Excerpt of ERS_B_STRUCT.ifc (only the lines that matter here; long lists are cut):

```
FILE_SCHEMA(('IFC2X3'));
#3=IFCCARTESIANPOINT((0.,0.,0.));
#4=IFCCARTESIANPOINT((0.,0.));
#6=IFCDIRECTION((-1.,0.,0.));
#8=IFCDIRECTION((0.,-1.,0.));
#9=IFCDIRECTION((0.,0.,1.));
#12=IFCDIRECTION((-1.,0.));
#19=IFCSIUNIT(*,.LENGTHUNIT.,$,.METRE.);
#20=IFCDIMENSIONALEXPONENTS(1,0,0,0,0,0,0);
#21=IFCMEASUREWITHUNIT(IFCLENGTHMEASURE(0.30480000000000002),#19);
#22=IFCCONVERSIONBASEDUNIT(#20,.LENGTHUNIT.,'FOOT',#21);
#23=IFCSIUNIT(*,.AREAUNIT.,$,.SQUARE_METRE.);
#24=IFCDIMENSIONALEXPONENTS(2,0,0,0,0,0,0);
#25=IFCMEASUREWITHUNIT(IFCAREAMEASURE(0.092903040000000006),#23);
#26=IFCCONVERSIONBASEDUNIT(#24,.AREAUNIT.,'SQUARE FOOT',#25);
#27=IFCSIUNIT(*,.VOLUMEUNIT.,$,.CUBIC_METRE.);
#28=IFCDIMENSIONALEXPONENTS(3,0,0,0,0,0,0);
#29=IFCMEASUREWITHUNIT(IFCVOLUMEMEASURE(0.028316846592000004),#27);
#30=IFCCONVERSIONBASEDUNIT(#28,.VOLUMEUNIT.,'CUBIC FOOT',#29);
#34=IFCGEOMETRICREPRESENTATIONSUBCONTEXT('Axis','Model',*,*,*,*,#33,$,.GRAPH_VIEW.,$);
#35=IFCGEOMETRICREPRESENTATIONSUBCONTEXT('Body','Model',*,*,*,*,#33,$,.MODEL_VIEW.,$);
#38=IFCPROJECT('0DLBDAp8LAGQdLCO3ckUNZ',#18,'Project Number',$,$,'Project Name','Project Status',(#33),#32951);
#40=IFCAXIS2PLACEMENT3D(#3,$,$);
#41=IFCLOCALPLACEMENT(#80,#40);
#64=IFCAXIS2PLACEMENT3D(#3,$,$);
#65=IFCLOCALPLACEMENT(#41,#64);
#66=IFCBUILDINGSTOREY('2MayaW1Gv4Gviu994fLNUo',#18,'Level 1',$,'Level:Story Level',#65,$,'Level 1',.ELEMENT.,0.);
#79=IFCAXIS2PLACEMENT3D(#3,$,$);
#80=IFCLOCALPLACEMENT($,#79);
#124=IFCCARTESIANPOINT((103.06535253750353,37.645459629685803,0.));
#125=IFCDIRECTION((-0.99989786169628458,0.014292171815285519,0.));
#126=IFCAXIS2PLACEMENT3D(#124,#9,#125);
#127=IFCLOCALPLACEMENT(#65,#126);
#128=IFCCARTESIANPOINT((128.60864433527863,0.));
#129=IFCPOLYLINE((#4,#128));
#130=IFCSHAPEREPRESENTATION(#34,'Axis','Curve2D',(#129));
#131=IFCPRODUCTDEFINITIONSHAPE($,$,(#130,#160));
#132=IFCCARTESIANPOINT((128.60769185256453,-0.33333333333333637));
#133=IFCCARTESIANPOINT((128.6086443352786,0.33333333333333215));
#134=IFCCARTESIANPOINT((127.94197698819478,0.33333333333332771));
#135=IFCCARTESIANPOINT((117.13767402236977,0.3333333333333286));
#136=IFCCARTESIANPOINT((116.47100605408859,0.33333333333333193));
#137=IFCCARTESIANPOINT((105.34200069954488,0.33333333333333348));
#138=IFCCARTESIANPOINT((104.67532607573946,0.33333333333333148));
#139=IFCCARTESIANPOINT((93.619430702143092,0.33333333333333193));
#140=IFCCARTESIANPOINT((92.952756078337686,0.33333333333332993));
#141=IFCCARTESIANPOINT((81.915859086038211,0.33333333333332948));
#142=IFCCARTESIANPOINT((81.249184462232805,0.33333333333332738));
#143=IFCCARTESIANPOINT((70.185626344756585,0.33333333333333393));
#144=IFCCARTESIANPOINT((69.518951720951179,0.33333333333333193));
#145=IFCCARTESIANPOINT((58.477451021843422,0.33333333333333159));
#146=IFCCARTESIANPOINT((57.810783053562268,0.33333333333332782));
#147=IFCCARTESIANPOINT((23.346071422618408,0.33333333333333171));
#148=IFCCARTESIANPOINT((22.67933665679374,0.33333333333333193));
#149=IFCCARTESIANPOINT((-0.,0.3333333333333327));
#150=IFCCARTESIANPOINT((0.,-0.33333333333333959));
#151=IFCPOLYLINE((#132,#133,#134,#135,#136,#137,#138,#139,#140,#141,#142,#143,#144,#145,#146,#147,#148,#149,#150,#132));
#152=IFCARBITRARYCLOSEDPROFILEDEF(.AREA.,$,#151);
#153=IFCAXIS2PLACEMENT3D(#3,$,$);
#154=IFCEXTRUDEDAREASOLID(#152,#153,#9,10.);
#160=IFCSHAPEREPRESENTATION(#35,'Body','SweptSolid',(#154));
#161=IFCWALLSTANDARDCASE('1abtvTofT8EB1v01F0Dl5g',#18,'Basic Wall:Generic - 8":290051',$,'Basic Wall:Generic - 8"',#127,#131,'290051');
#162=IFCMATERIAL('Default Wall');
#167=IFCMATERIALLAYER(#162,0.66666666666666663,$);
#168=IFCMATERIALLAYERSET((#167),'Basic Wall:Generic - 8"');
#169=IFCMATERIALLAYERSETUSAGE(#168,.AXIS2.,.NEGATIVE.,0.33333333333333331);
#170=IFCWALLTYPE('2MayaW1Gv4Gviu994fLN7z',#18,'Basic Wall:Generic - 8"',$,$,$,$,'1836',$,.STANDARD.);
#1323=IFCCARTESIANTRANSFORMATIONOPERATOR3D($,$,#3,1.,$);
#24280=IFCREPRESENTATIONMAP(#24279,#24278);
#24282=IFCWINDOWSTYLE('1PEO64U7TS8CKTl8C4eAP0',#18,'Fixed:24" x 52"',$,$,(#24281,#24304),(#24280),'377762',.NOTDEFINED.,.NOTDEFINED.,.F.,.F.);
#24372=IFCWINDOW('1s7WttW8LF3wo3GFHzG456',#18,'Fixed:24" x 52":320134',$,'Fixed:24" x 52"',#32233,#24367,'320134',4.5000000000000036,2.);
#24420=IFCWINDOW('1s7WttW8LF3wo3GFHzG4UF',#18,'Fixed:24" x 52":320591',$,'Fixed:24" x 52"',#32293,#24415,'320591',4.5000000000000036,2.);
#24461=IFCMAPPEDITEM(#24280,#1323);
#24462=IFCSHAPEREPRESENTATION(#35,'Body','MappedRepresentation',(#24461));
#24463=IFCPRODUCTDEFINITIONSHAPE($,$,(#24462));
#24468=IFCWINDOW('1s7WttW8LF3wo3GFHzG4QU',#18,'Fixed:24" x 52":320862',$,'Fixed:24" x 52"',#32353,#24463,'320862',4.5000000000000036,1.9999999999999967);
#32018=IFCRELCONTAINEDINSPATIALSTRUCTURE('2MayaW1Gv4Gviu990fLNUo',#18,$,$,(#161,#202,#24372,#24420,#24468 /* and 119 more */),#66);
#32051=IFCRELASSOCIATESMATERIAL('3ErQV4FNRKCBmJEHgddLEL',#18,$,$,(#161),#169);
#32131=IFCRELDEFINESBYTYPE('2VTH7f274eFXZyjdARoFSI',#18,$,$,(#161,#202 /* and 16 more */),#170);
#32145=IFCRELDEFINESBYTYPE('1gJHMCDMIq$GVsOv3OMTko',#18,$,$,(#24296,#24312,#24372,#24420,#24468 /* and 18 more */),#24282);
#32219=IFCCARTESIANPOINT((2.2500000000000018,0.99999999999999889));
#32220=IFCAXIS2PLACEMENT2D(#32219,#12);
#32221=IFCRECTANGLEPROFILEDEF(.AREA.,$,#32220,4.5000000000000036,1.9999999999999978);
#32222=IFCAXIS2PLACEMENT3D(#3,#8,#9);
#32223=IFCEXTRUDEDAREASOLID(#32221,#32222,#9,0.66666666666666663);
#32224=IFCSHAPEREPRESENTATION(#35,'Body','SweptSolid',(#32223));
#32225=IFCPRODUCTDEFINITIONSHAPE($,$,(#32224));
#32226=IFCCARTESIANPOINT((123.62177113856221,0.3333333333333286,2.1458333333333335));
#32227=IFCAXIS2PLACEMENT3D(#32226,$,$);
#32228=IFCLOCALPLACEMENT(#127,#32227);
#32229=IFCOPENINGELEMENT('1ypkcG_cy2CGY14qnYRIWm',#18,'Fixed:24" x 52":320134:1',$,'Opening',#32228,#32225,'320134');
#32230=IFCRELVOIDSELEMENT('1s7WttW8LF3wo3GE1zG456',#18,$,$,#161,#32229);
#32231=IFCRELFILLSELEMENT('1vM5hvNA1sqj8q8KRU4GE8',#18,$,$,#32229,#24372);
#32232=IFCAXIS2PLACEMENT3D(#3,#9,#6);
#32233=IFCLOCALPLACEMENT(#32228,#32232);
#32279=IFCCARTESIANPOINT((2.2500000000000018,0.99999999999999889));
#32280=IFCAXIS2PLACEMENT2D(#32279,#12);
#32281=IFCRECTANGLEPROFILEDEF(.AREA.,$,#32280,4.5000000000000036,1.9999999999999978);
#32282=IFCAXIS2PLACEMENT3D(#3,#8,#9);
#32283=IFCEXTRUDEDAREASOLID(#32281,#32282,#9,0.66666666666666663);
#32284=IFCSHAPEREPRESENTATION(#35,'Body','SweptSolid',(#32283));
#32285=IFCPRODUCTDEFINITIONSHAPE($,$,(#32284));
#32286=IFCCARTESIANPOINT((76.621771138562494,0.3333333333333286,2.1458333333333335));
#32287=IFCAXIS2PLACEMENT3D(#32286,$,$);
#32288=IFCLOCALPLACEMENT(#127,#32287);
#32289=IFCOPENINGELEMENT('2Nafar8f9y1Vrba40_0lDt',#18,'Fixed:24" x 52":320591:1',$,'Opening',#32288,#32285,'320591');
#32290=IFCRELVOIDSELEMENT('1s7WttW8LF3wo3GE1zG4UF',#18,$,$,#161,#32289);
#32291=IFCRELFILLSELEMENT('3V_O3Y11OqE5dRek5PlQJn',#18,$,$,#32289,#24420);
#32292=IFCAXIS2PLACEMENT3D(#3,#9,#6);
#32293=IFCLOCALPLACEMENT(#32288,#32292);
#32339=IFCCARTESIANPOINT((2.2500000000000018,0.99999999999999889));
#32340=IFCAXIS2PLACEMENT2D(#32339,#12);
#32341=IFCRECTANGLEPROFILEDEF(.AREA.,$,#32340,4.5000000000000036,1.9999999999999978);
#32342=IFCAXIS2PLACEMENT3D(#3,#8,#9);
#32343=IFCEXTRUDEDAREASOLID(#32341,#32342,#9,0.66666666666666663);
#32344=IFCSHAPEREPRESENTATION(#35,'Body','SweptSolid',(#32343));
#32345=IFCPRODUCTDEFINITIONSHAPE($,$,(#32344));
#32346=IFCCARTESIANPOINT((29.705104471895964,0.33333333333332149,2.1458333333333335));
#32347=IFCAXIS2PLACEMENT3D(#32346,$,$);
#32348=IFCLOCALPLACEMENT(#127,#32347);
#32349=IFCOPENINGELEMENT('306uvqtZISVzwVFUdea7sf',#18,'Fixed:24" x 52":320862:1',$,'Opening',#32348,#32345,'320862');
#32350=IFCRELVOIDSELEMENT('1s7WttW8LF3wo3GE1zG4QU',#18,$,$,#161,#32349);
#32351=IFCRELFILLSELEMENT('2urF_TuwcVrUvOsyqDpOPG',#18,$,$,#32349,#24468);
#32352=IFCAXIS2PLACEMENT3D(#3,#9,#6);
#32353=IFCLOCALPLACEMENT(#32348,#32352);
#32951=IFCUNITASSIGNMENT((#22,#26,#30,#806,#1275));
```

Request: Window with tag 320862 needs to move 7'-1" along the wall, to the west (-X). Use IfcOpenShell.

```python
import ifcopenshell
import ifcopenshell.api.geometry
import ifcopenshell.util.placement
import ifcopenshell.util.unit

model = ifcopenshell.open("ERS_B_STRUCT.ifc")
unit_scale = ifcopenshell.util.unit.calculate_unit_scale(model)

window = model.by_guid("1s7WttW8LF3wo3GFHzG4QU")
opening = window.FillsVoids[0].RelatingOpeningElement
wall = opening.VoidsElements[0].RelatingBuildingElement

wall_matrix = ifcopenshell.util.placement.get_local_placement(wall.ObjectPlacement)
shift = wall_matrix[:3, 0] * 85 * 0.0254 / unit_scale
before = ifcopenshell.util.placement.get_local_placement(window.ObjectPlacement)[:3, 3].copy()

# The window is placed relative to its opening, so it follows when the opening moves.
matrix = ifcopenshell.util.placement.get_local_placement(opening.ObjectPlacement)
matrix[:3, 3] += shift
ifcopenshell.api.geometry.edit_object_placement(
    model, product=opening, matrix=matrix, is_si=False, should_transform_children=True
)

after = ifcopenshell.util.placement.get_local_placement(window.ObjectPlacement)[:3, 3]
print("window moved by", (after - before).round(3) + 0.0)

model.write("ERS_B_STRUCT-out.ifc")
```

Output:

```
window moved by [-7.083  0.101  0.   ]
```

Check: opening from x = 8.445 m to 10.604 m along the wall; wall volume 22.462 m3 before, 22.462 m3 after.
